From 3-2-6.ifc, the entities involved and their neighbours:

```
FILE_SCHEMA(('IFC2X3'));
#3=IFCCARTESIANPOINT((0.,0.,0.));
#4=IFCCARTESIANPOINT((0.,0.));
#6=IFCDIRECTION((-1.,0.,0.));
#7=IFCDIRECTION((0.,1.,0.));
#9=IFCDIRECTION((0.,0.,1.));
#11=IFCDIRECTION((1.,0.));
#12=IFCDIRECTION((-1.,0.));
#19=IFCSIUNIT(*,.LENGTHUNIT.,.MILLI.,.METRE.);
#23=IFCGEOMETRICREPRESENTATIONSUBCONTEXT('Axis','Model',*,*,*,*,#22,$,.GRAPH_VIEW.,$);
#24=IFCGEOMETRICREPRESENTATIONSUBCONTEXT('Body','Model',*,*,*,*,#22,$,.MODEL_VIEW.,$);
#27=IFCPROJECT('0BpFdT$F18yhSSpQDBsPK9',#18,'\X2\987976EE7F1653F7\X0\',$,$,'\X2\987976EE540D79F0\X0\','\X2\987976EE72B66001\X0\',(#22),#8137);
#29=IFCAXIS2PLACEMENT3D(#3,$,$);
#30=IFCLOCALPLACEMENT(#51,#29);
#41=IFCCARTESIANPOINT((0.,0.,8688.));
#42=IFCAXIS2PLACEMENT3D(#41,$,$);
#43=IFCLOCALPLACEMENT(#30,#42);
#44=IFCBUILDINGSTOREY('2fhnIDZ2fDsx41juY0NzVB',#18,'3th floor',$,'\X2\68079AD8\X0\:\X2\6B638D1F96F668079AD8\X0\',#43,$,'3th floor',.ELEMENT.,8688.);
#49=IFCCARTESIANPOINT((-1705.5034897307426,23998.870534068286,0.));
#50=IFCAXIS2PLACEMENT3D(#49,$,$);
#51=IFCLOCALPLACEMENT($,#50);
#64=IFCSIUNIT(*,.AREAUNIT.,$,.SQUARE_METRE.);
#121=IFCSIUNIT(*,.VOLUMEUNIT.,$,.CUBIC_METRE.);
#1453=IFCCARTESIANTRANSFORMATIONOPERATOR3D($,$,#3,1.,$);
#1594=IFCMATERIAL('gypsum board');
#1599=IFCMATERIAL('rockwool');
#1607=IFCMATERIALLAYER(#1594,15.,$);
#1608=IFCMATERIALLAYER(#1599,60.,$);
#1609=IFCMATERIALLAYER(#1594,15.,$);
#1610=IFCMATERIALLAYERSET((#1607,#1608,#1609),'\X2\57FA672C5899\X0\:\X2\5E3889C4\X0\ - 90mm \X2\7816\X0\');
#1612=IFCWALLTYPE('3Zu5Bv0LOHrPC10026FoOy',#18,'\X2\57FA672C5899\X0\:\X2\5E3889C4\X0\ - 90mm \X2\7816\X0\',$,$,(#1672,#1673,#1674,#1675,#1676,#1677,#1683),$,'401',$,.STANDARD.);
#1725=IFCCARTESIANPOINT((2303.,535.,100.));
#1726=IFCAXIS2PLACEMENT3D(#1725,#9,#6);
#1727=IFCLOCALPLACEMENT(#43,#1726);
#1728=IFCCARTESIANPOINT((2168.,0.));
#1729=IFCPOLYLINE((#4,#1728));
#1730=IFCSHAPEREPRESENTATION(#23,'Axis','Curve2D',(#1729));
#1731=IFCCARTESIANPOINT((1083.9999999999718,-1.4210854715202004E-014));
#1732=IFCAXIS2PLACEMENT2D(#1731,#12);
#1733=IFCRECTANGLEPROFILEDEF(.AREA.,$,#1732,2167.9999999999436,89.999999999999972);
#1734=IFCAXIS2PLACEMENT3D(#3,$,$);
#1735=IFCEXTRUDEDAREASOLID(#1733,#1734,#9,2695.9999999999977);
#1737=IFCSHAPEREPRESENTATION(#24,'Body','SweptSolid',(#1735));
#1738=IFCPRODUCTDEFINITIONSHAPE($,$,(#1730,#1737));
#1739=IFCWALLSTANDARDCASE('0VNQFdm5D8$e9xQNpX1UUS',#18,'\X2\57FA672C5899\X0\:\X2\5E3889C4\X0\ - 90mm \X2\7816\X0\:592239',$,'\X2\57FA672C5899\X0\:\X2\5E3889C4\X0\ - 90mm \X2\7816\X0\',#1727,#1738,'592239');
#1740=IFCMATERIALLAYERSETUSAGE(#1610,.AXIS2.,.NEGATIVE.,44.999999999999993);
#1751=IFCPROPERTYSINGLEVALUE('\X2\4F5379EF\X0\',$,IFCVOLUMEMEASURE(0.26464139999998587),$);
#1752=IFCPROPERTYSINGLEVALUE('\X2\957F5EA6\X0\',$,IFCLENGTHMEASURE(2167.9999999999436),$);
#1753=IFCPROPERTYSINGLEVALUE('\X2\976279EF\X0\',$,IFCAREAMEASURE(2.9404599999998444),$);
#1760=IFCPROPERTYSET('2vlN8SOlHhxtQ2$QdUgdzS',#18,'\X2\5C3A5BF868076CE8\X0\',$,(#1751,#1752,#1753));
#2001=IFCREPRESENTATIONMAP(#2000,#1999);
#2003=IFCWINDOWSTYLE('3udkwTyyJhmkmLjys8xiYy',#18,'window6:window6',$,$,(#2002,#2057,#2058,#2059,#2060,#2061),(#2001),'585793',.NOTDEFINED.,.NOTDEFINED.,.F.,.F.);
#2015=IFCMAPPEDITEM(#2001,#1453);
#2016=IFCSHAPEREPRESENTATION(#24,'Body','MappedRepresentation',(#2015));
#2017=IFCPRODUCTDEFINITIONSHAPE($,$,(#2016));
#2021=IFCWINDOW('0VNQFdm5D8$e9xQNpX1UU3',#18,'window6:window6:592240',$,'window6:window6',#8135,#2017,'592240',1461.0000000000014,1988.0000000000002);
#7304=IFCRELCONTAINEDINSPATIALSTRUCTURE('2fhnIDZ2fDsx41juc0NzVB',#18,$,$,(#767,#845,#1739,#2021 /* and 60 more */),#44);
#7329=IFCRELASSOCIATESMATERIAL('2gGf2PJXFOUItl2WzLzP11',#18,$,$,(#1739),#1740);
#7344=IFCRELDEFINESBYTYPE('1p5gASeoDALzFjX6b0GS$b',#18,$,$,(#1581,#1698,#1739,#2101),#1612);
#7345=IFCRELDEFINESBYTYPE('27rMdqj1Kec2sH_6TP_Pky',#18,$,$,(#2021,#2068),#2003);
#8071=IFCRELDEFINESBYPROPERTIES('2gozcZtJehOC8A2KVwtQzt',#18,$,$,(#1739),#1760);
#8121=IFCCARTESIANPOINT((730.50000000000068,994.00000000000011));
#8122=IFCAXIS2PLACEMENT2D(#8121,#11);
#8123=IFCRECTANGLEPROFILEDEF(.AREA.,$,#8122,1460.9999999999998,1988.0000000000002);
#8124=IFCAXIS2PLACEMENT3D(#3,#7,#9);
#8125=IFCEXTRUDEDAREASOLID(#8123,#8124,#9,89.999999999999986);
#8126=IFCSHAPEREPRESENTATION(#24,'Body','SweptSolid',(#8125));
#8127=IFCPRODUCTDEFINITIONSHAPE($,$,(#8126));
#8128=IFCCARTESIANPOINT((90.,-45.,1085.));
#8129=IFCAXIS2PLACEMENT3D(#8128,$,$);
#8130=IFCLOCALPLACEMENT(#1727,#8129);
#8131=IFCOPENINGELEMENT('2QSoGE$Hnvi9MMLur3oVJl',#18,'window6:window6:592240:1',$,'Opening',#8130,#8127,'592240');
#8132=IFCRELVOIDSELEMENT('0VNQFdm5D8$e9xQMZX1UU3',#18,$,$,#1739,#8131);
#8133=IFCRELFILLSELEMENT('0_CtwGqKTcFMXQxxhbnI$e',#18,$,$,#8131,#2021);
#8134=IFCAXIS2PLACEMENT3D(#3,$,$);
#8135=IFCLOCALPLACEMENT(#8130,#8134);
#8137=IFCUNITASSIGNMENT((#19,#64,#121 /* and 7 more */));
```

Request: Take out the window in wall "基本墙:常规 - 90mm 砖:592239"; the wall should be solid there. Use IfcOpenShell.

```python
import ifcopenshell
import ifcopenshell.api.feature
import ifcopenshell.api.pset
import ifcopenshell.api.root
import ifcopenshell.geom
import ifcopenshell.util.element
import ifcopenshell.util.shape
import ifcopenshell.util.unit

model = ifcopenshell.open("3-2-6.ifc")
area_scale = ifcopenshell.util.unit.calculate_unit_scale(model, "AREAUNIT")
volume_scale = ifcopenshell.util.unit.calculate_unit_scale(model, "VOLUMEUNIT")
settings = ifcopenshell.geom.settings()


def volume(element):
    """Net volume in cubic metres, openings subtracted."""
    shape = ifcopenshell.geom.create_shape(settings, element)
    return ifcopenshell.util.shape.get_volume(shape.geometry)


window = model.by_guid("0VNQFdm5D8$e9xQNpX1UU3")
opening = window.FillsVoids[0].RelatingOpeningElement
wall = opening.VoidsElements[0].RelatingBuildingElement
before = volume(wall)

ifcopenshell.api.root.remove_product(model, product=window)
ifcopenshell.api.feature.remove_feature(model, feature=opening)

after = volume(wall)
thickness = 0.09  # wall thickness in metres

# Update the wall's stored quantities.
pset = model.by_id(ifcopenshell.util.element.get_pset(wall, "尺寸标注", should_inherit=False)["id"])
ifcopenshell.api.pset.edit_pset(model, pset=pset, properties={
    "体积": model.create_entity("IfcVolumeMeasure", after / volume_scale),
    "面积": model.create_entity("IfcAreaMeasure", after / thickness / area_scale),
})

print(f"wall volume {before:.3f} -> {after:.3f} m3")

model.write("3-2-6_edited.ifc")
```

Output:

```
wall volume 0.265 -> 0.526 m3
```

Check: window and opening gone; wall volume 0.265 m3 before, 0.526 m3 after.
